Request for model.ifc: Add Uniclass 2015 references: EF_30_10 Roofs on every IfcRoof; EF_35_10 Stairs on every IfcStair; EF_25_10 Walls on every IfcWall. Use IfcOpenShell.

First a look at what the model holds.

```python
import ifcopenshell

model = ifcopenshell.open("model.ifc")
print(model.schema)
print("classifications:", [c.Name for c in model.by_type("IfcClassification")])
for ifc_class in ("IfcDoor", "IfcRoof", "IfcStair", "IfcWall", "IfcWindow"):
    print(ifc_class, len(model.by_type(ifc_class)))
```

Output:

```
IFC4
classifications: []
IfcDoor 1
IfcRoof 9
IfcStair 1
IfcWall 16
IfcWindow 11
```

```python
import ifcopenshell
import ifcopenshell.api.classification

model = ifcopenshell.open("model.ifc")

system = ifcopenshell.api.classification.add_classification(model, classification="Uniclass 2015")

codes = {
    "IfcRoof": ("EF_30_10", "Roofs"),
    "IfcStair": ("EF_35_10", "Stairs"),
    "IfcWall": ("EF_25_10", "Walls"),
}
for ifc_class, (code, name) in codes.items():
    products = model.by_type(ifc_class)
    ifcopenshell.api.classification.add_reference(
        model, products=products, classification=system, identification=code, name=name
    )
    print(code, len(products))

model.write("model-out.ifc")
```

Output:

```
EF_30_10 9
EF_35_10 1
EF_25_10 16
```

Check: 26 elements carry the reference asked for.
